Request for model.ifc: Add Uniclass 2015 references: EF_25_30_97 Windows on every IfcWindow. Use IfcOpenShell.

First a look at what the model holds.

```python
import ifcopenshell

model = ifcopenshell.open("model.ifc")
print(model.schema)
print("classifications:", [c.Name for c in model.by_type("IfcClassification")])
for ifc_class in ("IfcDoor", "IfcRoof", "IfcStair", "IfcWall", "IfcWindow"):
    print(ifc_class, len(model.by_type(ifc_class)))
```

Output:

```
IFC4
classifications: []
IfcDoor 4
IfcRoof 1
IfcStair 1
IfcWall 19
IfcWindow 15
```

```python
import ifcopenshell
import ifcopenshell.api.classification

model = ifcopenshell.open("model.ifc")

system = ifcopenshell.api.classification.add_classification(model, classification="Uniclass 2015")

codes = {
    "IfcWindow": ("EF_25_30_97", "Windows"),
}
for ifc_class, (code, name) in codes.items():
    products = model.by_type(ifc_class)
    ifcopenshell.api.classification.add_reference(
        model, products=products, classification=system, identification=code, name=name
    )
    print(code, len(products))

model.write("model_v2.ifc")
```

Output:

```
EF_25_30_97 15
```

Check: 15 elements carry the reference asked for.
